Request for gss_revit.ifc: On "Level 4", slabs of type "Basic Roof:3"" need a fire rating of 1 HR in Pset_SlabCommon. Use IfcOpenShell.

First a look at what the model holds.

```python
import ifcopenshell
import ifcopenshell.util.element

model = ifcopenshell.open("gss_revit.ifc")
print(model.schema)
storey = next(s for s in model.by_type("IfcBuildingStorey") if s.Name == "Level 4")
slabs = [e for e in ifcopenshell.util.element.get_decomposition(storey) if e.is_a("IfcSlab")]
seen = {}
for e in slabs:
    element_type = ifcopenshell.util.element.get_type(e)
    key = (element_type.Name if element_type != e and element_type else None, ifcopenshell.util.element.get_pset(e, "Pset_SlabCommon", "FireRating"))
    seen[key] = seen.get(key, 0) + 1
for (name, value), count in sorted(seen.items(), key=str):
    print(count, "x", name, "|", value)
```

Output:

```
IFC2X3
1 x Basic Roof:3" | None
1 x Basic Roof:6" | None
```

```python
import ifcopenshell
import ifcopenshell.api.pset
import ifcopenshell.util.element

model = ifcopenshell.open("gss_revit.ifc")

storey = next(s for s in model.by_type("IfcBuildingStorey") if s.Name == "Level 4")
slabs = [e for e in ifcopenshell.util.element.get_decomposition(storey) if e.is_a("IfcSlab")]

count = 0
for e in slabs:
    element_type = ifcopenshell.util.element.get_type(e)
    if element_type in (None, e) or element_type.Name != 'Basic Roof:3"':
        continue
    # add_pset returns the element's existing set when there is one.
    pset = ifcopenshell.api.pset.add_pset(model, product=e, name="Pset_SlabCommon")
    ifcopenshell.api.pset.edit_pset(model, pset=pset, properties={"FireRating": "1 HR"})
    count += 1

print(count, "slabs updated")

model.write("gss_revit_edited.ifc")
```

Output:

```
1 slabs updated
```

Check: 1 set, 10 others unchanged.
